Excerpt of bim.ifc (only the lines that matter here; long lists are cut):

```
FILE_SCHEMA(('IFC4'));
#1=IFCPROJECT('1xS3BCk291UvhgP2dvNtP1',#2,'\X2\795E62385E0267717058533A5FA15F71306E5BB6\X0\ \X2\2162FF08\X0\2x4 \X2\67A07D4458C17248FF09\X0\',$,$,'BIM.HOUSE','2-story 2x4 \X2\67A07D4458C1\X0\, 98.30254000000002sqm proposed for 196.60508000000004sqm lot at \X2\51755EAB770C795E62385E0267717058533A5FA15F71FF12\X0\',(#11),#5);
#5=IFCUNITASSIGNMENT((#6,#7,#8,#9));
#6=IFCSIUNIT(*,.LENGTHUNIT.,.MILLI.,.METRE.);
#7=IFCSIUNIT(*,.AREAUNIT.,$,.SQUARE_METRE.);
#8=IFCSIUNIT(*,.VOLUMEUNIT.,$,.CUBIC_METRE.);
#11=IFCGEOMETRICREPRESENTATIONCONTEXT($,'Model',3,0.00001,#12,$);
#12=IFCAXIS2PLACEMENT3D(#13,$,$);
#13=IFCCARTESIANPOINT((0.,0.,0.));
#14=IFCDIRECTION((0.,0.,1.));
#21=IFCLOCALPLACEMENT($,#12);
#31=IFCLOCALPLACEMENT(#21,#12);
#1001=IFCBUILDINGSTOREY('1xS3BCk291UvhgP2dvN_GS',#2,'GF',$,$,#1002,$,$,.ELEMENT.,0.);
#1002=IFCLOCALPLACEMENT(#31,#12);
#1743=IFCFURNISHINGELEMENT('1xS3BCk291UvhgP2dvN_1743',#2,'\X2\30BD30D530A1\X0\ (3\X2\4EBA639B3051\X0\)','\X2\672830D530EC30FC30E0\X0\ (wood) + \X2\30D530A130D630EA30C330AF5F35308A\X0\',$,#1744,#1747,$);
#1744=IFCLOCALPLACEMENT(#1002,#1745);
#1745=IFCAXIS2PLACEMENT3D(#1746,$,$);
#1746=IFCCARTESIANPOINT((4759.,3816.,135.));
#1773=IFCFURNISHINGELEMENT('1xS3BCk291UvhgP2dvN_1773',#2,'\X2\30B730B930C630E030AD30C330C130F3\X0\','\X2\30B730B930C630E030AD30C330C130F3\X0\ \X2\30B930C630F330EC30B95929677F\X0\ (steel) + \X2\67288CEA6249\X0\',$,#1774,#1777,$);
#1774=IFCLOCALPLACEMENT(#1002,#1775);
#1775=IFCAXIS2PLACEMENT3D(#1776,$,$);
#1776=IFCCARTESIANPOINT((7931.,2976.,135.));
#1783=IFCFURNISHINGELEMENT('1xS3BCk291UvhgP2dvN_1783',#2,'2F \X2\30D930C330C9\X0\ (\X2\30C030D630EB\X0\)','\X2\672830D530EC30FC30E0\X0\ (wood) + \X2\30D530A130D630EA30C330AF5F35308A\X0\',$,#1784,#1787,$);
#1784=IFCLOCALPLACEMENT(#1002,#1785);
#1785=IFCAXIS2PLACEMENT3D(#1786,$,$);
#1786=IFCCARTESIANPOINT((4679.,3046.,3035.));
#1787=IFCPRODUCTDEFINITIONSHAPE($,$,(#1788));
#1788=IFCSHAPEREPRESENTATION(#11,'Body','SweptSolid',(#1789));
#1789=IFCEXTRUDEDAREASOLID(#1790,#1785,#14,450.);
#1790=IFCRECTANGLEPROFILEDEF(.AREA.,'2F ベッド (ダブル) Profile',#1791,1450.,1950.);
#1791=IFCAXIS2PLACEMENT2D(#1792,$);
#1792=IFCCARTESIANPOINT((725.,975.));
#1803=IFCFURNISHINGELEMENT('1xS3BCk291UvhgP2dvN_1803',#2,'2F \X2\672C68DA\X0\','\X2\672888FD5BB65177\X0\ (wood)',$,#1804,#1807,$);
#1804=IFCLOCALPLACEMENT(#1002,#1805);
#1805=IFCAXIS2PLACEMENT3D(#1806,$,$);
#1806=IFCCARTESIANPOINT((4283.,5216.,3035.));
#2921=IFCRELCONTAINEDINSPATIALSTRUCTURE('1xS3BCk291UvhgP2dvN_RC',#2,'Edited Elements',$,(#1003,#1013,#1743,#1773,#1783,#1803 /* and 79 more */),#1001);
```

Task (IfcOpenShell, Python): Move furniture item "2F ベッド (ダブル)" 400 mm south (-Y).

```python
import ifcopenshell
import ifcopenshell.api.geometry
import ifcopenshell.util.placement
import ifcopenshell.util.unit

model = ifcopenshell.open("bim.ifc")
unit_scale = ifcopenshell.util.unit.calculate_unit_scale(model)

item = model.by_guid("1xS3BCk291UvhgP2dvN_1783")
matrix = ifcopenshell.util.placement.get_local_placement(item.ObjectPlacement)
matrix[1, 3] -= 0.4 / unit_scale
ifcopenshell.api.geometry.edit_object_placement(model, product=item, matrix=matrix, is_si=False)

print(ifcopenshell.util.placement.get_local_placement(item.ObjectPlacement).round(3) + 0.0)

model.write("bim_v2.ifc")
```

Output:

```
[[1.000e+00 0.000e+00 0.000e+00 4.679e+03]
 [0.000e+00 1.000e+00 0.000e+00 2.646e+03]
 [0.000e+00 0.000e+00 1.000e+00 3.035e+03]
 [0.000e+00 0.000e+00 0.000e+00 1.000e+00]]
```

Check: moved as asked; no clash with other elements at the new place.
